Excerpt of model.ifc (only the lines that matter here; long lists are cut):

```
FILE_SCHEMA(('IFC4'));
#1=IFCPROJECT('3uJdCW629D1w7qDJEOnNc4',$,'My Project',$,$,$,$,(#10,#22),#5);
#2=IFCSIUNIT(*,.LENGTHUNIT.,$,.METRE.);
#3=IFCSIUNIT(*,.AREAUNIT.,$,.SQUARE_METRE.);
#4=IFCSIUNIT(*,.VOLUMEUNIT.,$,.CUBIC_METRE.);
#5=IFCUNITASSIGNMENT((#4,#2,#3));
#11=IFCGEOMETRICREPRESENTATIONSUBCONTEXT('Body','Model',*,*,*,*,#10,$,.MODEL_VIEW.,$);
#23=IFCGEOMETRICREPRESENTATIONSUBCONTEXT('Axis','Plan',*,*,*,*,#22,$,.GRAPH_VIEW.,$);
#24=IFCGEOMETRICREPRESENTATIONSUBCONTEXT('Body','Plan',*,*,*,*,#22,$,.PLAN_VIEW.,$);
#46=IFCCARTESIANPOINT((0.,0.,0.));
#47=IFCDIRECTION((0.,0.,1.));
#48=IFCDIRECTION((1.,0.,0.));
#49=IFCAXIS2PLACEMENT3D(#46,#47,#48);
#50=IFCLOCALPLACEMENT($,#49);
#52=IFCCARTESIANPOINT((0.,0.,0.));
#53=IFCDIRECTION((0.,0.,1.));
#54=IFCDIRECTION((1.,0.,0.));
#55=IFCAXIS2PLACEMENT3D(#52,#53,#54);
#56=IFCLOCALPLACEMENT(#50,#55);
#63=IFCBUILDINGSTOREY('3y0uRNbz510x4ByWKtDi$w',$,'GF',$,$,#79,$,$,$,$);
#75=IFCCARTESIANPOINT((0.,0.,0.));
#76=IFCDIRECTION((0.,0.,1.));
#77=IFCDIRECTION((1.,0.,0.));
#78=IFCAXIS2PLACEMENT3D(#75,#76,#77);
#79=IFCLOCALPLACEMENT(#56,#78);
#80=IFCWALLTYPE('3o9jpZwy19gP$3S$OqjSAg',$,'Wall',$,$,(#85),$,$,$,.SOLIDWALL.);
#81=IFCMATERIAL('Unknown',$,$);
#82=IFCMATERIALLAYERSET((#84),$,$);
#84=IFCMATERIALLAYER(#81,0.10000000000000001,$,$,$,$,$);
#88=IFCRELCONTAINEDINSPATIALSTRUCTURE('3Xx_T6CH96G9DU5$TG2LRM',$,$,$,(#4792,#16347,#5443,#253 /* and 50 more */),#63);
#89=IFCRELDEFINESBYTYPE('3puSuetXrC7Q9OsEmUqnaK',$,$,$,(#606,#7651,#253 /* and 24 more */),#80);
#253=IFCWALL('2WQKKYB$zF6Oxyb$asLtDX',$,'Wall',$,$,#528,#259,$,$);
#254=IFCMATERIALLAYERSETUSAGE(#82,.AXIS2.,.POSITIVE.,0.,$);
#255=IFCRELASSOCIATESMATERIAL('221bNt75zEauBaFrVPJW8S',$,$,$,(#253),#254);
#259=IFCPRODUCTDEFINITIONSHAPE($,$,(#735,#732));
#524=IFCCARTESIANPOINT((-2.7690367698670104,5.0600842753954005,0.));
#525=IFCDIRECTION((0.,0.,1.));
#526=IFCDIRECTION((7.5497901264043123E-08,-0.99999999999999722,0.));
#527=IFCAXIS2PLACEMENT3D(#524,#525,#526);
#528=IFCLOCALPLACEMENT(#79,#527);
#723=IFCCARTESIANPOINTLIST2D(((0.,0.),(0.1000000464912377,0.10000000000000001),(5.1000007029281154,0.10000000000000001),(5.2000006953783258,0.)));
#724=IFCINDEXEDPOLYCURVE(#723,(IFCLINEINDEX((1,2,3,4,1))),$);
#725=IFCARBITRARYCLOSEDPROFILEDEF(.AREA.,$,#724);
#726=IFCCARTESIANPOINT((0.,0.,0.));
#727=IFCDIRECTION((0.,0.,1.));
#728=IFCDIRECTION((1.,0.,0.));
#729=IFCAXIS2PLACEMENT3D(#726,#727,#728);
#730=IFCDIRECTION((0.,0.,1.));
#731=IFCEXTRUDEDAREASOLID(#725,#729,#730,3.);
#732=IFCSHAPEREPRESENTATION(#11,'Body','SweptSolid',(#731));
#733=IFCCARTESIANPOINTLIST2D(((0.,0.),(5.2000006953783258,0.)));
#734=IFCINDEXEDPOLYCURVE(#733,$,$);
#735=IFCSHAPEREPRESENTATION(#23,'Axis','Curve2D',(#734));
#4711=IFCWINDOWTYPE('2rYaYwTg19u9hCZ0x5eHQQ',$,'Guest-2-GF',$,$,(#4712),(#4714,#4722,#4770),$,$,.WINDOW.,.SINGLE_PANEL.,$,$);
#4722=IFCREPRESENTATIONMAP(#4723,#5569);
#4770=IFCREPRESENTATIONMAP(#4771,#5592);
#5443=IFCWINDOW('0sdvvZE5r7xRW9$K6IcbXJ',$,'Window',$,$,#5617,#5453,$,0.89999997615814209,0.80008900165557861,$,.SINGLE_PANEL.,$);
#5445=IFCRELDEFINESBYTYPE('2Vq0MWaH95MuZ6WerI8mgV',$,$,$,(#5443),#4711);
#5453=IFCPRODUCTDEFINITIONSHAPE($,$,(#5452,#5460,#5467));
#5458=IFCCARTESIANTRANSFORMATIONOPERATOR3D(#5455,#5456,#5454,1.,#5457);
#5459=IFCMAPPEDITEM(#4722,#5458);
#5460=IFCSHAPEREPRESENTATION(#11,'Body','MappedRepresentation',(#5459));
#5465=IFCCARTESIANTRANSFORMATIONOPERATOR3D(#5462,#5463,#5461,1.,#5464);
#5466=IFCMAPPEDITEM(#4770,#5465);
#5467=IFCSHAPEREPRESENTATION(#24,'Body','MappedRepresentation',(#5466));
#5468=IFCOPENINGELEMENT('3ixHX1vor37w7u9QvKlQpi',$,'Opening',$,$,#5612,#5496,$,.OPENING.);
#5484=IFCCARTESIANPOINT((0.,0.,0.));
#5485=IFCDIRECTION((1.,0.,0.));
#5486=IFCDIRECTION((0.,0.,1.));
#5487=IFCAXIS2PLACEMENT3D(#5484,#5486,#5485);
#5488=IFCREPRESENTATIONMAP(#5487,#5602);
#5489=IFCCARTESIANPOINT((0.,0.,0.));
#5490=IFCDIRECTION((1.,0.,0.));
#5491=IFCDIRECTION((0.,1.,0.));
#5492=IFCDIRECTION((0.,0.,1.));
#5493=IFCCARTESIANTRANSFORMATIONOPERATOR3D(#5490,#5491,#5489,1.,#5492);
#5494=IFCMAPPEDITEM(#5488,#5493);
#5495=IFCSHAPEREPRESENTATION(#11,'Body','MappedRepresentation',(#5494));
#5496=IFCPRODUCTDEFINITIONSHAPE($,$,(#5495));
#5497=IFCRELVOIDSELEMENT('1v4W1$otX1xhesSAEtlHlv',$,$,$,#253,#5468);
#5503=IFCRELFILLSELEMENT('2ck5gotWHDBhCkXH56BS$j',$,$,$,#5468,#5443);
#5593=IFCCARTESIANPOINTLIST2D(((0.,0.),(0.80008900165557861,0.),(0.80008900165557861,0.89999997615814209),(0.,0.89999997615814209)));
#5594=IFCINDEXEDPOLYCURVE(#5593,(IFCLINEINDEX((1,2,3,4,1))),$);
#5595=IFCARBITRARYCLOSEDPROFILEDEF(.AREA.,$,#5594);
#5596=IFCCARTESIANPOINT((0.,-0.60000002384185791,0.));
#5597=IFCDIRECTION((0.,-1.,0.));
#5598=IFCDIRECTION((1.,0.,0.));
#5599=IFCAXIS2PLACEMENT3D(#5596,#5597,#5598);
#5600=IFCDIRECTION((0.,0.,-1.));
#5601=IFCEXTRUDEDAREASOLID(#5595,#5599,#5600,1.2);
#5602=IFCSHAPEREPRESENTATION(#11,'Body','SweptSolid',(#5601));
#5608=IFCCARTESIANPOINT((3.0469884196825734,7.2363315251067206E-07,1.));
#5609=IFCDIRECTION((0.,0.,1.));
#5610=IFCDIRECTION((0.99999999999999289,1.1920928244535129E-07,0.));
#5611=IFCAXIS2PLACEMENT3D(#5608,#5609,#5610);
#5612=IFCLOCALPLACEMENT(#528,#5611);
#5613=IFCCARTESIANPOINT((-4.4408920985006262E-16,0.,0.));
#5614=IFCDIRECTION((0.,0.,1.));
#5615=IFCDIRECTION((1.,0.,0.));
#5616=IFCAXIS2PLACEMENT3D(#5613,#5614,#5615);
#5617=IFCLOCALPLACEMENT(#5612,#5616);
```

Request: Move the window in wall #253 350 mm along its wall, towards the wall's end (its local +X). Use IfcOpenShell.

```python
import ifcopenshell
import ifcopenshell.api.geometry
import ifcopenshell.util.placement
import ifcopenshell.util.unit

model = ifcopenshell.open("model.ifc")
unit_scale = ifcopenshell.util.unit.calculate_unit_scale(model)

window = model.by_guid("0sdvvZE5r7xRW9$K6IcbXJ")
opening = window.FillsVoids[0].RelatingOpeningElement
wall = opening.VoidsElements[0].RelatingBuildingElement

wall_matrix = ifcopenshell.util.placement.get_local_placement(wall.ObjectPlacement)
shift = wall_matrix[:3, 0] * 0.35 / unit_scale
before = ifcopenshell.util.placement.get_local_placement(window.ObjectPlacement)[:3, 3].copy()

# The window is placed relative to its opening, so it follows when the opening moves.
matrix = ifcopenshell.util.placement.get_local_placement(opening.ObjectPlacement)
matrix[:3, 3] += shift
ifcopenshell.api.geometry.edit_object_placement(
    model, product=opening, matrix=matrix, is_si=False, should_transform_children=True
)

after = ifcopenshell.util.placement.get_local_placement(window.ObjectPlacement)[:3, 3]
print("window moved by", (after - before).round(3) + 0.0)

model.write("model_updated.ifc")
```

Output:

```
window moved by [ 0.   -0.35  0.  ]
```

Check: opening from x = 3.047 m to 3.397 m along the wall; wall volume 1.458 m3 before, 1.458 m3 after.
